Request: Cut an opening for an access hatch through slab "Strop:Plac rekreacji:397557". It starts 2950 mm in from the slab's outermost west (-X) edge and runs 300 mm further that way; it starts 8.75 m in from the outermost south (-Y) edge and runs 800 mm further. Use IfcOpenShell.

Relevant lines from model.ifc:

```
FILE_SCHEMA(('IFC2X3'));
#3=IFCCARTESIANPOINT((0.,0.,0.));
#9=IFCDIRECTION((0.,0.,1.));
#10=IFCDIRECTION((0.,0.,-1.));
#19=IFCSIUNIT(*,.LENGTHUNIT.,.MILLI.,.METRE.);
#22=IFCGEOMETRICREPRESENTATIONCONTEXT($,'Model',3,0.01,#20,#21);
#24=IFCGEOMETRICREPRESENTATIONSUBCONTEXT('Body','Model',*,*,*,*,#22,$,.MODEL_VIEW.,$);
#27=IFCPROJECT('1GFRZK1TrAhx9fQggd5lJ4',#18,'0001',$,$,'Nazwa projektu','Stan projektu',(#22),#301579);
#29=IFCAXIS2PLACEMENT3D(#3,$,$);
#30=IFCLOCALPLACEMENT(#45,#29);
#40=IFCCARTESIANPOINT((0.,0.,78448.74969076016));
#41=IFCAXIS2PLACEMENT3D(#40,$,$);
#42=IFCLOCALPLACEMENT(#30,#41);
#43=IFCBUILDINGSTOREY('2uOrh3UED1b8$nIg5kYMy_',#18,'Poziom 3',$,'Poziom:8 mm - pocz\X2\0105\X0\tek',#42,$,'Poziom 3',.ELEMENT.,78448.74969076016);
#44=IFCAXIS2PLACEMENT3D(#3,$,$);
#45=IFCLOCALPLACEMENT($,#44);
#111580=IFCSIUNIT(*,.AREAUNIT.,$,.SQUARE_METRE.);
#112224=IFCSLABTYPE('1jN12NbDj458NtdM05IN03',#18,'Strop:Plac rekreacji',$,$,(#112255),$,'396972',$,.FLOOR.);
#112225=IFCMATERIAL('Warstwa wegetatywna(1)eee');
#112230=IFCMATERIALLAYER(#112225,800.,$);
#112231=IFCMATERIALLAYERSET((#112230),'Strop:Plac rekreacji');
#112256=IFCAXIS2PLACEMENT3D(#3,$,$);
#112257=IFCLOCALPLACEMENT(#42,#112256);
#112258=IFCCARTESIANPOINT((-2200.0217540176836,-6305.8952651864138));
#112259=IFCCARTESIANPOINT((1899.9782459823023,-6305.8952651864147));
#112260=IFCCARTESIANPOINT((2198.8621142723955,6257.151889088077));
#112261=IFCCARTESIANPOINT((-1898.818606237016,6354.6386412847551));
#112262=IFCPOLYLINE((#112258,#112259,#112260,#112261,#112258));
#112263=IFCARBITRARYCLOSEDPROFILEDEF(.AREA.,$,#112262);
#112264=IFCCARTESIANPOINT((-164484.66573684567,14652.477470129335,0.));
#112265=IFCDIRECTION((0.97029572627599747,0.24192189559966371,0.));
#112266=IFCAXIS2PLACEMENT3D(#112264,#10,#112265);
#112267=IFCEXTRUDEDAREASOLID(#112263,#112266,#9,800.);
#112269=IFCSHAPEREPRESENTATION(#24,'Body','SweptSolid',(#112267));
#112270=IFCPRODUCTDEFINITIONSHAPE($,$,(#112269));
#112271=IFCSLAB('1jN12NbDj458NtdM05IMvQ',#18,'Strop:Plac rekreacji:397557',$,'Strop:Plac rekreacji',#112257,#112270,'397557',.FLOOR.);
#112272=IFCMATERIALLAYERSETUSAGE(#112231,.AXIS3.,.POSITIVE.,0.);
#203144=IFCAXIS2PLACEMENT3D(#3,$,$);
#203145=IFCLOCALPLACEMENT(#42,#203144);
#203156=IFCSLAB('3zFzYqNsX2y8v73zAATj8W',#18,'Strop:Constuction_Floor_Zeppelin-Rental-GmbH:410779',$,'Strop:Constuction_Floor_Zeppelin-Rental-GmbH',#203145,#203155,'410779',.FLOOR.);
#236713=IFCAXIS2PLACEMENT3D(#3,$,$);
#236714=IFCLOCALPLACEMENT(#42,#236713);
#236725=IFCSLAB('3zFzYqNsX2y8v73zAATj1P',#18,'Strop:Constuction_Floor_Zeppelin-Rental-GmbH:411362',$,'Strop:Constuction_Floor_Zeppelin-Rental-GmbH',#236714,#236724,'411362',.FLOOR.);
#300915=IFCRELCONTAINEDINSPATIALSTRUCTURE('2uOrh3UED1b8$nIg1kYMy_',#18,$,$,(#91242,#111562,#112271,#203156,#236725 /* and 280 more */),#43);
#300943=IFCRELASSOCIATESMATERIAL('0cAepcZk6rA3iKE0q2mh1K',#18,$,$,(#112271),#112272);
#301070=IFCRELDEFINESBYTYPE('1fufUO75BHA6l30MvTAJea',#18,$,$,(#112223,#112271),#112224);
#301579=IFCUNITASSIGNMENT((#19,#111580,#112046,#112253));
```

```python
import numpy as np
import ifcopenshell
import ifcopenshell.api.feature
import ifcopenshell.api.geometry
import ifcopenshell.api.root
import ifcopenshell.geom
import ifcopenshell.util.placement
import ifcopenshell.util.representation
import ifcopenshell.util.shape
import ifcopenshell.util.unit

model = ifcopenshell.open("model.ifc")
unit_scale = ifcopenshell.util.unit.calculate_unit_scale(model)
settings = ifcopenshell.geom.settings()


def volume(element):
    """Net volume in cubic metres, openings subtracted."""
    shape = ifcopenshell.geom.create_shape(settings, element)
    return ifcopenshell.util.shape.get_volume(shape.geometry)


slab = model.by_guid("1jN12NbDj458NtdM05IMvQ")
before = volume(slab)

# Extent in the slab's own axes, in metres. The edges named are its -X and -Y sides.
slab_shape = ifcopenshell.geom.create_shape(settings, slab)
vertices = ifcopenshell.util.shape.get_vertices(slab_shape.geometry)
x_min, y_min, bottom = vertices.min(axis=0)
top = vertices[:, 2].max()

opening = ifcopenshell.api.root.create_entity(model, ifc_class="IfcOpeningElement", name="Access hatch opening")
context = ifcopenshell.util.representation.get_context(model, "Model", "Body", "MODEL_VIEW")
width, depth = 0.3, 0.8
outline = [(0.0, 0.0), (width, 0.0), (width, depth), (0.0, depth), (0.0, 0.0)]
# Overshoot both faces by 50 mm so the cut is clean.
shape = ifcopenshell.api.geometry.add_slab_representation(
    model, context=context, depth=top - bottom + 0.1, polyline=outline
)
ifcopenshell.api.geometry.assign_representation(model, product=opening, representation=shape)

matrix = ifcopenshell.util.placement.get_local_placement(slab.ObjectPlacement)
matrix[:, 3] = matrix @ np.append(np.array([x_min + 2.95, y_min + 8.75, bottom - 0.05]) / unit_scale, 1.0)
ifcopenshell.api.geometry.edit_object_placement(model, product=opening, matrix=matrix, is_si=False)
ifcopenshell.api.feature.add_feature(model, feature=opening, element=slab)

after = volume(slab)

print(f"slab volume {before:.3f} -> {after:.3f} m3")

model.write("model_rev.ifc")
```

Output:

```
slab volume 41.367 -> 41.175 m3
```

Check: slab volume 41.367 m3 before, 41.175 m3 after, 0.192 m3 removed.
